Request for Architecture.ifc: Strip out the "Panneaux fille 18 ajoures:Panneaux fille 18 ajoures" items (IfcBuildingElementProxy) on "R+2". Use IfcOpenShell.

First a look at what the model holds.

```python
import ifcopenshell
import ifcopenshell.util.element

model = ifcopenshell.open("Architecture.ifc")
print(model.schema)
storey = next(s for s in model.by_type("IfcBuildingStorey") if s.Name == "R+2")
proxies = [e for e in ifcopenshell.util.element.get_decomposition(storey) if e.is_a("IfcBuildingElementProxy")]
seen = {}
for e in proxies:
    element_type = ifcopenshell.util.element.get_type(e)
    name = element_type.Name if element_type not in (None, e) else None
    seen[name] = seen.get(name, 0) + 1
for name, count in sorted(seen.items(), key=str):
    print(count, "x", name)
```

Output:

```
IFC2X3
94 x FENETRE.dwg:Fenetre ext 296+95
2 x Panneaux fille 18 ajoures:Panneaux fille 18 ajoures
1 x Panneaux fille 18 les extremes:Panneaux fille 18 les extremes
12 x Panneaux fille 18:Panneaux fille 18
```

```python
import ifcopenshell
import ifcopenshell.api.root
import ifcopenshell.util.element

model = ifcopenshell.open("Architecture.ifc")

storey = next(s for s in model.by_type("IfcBuildingStorey") if s.Name == "R+2")
proxies = [e for e in ifcopenshell.util.element.get_decomposition(storey) if e.is_a("IfcBuildingElementProxy")]
targets = [e for e in proxies if (t := ifcopenshell.util.element.get_type(e)) not in (None, e) and t.Name == "Panneaux fille 18 ajoures:Panneaux fille 18 ajoures"]

for e in targets:
    ifcopenshell.api.root.remove_product(model, product=e)
print(len(targets), "removed")

model.write("Architecture_updated.ifc")
```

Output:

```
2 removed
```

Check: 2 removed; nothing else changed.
